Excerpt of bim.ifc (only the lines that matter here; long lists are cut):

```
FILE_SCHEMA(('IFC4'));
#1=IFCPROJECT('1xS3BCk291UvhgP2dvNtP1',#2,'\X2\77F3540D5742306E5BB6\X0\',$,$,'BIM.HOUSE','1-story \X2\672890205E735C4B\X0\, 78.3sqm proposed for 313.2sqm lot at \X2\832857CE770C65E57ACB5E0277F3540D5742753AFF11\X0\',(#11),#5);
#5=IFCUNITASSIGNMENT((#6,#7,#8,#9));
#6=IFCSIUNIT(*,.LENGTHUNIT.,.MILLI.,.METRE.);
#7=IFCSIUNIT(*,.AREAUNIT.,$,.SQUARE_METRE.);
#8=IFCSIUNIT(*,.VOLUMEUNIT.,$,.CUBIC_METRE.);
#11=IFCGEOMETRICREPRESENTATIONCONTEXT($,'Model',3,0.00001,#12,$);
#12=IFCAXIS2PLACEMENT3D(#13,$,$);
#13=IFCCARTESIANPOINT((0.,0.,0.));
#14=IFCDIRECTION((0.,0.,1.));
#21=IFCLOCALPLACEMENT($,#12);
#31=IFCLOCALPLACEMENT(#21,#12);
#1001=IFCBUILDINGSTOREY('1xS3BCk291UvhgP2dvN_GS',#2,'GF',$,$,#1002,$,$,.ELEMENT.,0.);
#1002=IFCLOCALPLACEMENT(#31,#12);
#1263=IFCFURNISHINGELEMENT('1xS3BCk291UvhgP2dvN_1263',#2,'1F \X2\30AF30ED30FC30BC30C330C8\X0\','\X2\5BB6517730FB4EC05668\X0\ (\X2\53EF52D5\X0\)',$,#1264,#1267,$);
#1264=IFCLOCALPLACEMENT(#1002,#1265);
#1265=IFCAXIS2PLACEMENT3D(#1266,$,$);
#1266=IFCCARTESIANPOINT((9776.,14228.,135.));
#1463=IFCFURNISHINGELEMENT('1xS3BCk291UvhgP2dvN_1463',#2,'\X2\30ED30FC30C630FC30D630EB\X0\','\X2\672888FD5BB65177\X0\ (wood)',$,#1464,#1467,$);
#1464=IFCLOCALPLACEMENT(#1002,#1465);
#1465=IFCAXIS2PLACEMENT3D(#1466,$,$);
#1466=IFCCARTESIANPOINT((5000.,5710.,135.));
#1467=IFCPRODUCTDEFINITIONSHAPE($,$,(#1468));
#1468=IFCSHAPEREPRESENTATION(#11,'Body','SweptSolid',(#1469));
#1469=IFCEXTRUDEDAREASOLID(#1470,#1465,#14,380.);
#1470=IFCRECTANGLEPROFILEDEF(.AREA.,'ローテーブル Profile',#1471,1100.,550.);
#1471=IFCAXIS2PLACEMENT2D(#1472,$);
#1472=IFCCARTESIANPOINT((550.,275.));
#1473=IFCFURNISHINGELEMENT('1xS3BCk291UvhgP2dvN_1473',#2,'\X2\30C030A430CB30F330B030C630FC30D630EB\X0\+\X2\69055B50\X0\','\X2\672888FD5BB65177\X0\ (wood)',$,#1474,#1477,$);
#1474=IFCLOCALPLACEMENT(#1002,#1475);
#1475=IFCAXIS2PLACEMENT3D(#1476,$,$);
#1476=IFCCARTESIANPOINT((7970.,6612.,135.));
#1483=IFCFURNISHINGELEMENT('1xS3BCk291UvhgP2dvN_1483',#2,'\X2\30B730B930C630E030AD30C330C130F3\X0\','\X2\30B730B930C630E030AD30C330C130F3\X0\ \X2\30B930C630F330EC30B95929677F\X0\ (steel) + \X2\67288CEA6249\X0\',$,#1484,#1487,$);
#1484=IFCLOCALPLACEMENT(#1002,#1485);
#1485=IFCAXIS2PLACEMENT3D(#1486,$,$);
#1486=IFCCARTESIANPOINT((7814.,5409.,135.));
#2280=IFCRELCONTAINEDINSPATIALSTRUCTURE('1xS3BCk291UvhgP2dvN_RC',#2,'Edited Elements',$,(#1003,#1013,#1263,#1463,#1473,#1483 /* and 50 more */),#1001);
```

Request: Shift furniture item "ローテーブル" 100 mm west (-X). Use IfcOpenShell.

```python
import ifcopenshell
import ifcopenshell.api.geometry
import ifcopenshell.util.placement
import ifcopenshell.util.unit

model = ifcopenshell.open("bim.ifc")
unit_scale = ifcopenshell.util.unit.calculate_unit_scale(model)

item = model.by_guid("1xS3BCk291UvhgP2dvN_1463")
matrix = ifcopenshell.util.placement.get_local_placement(item.ObjectPlacement)
matrix[0, 3] -= 0.1 / unit_scale
ifcopenshell.api.geometry.edit_object_placement(model, product=item, matrix=matrix, is_si=False)

print(ifcopenshell.util.placement.get_local_placement(item.ObjectPlacement).round(3) + 0.0)

model.write("bim_v2.ifc")
```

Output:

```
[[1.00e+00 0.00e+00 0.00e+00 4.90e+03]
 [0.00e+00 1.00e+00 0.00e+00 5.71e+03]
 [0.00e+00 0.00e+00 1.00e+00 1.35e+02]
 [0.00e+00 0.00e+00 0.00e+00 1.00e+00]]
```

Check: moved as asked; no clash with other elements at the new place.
